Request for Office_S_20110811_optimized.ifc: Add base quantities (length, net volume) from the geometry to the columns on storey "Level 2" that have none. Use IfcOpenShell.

First a look at what the model holds.

```python
import ifcopenshell
import ifcopenshell.util.element
import ifcopenshell.util.unit

model = ifcopenshell.open("Office_S_20110811_optimized.ifc")
print(model.schema)
for unit_type in ("LENGTHUNIT", "AREAUNIT", "VOLUMEUNIT"):
    print(unit_type, ifcopenshell.util.unit.calculate_unit_scale(model, unit_type))
storey = next(s for s in model.by_type("IfcBuildingStorey") if s.Name == "Level 2")
columns = [e for e in ifcopenshell.util.element.get_decomposition(storey) if e.is_a("IfcColumn")]
for e in sorted(columns, key=lambda e: e.id()):
    print(e.id(), e.is_a(), e.Name, list(ifcopenshell.util.element.get_psets(e, qtos_only=True)), sep=" | ")
```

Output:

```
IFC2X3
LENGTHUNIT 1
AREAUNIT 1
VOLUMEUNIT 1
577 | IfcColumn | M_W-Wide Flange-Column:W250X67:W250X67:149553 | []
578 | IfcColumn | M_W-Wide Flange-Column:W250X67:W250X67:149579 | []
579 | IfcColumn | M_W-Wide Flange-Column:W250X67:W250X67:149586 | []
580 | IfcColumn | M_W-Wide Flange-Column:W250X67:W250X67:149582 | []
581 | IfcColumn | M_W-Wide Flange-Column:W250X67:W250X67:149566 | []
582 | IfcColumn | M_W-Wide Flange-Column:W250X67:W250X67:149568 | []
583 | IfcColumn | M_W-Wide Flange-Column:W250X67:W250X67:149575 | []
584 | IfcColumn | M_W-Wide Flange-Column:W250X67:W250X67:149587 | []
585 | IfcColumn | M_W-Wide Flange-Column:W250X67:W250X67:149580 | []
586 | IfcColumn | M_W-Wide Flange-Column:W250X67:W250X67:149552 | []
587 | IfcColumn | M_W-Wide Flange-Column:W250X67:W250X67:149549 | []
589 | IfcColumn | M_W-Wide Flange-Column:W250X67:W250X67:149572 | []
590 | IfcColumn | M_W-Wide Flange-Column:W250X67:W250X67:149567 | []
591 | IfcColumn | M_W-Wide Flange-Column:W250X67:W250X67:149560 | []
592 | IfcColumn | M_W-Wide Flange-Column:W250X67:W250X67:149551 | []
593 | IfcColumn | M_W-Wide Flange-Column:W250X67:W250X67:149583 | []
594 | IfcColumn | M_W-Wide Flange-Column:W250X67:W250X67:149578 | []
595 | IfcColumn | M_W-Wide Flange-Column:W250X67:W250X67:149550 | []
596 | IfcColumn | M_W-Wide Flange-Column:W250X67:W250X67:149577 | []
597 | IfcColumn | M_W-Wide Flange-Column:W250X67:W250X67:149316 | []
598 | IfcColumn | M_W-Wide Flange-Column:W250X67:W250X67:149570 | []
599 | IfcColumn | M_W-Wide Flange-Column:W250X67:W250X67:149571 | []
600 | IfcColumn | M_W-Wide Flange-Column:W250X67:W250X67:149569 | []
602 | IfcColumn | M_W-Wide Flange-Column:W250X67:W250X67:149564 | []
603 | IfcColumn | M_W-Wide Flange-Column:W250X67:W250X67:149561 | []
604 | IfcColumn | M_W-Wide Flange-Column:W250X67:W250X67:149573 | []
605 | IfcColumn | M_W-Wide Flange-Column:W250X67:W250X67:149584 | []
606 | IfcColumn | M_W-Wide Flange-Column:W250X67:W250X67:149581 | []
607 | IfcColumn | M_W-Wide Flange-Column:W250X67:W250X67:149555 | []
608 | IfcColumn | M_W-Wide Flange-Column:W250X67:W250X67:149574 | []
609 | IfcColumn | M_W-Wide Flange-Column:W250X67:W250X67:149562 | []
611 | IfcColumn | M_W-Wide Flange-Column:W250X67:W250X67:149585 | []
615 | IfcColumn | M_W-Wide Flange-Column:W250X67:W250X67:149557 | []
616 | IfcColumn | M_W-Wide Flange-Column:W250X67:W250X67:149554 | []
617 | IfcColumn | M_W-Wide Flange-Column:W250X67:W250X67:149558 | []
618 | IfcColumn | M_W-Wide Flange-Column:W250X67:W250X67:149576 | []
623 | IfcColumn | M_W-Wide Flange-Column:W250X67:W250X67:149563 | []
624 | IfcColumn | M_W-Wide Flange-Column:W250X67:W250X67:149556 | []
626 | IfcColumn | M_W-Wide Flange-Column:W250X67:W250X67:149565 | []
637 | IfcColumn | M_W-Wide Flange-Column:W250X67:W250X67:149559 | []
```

```python
import ifcopenshell
import ifcopenshell.api.pset
import ifcopenshell.geom
import ifcopenshell.util.element
import ifcopenshell.util.shape
import ifcopenshell.util.unit

model = ifcopenshell.open("Office_S_20110811_optimized.ifc")
unit_scale = ifcopenshell.util.unit.calculate_unit_scale(model)
volume_scale = ifcopenshell.util.unit.calculate_unit_scale(model, "VOLUMEUNIT")
settings = ifcopenshell.geom.settings()

storey = next(s for s in model.by_type("IfcBuildingStorey") if s.Name == "Level 2")
columns = [e for e in ifcopenshell.util.element.get_decomposition(storey) if e.is_a("IfcColumn")]

for e in sorted(columns, key=lambda e: e.id()):
    if ifcopenshell.util.element.get_psets(e, qtos_only=True, should_inherit=False):
        continue
    # Geometry comes back in metres, in the element's own axes.
    shape = ifcopenshell.geom.create_shape(settings, e)
    values = {
        "Length": ifcopenshell.util.shape.get_z(shape.geometry) / unit_scale,
        "NetVolume": ifcopenshell.util.shape.get_volume(shape.geometry) / volume_scale,
    }
    qto = ifcopenshell.api.pset.add_qto(model, product=e, name="BaseQuantities")
    ifcopenshell.api.pset.edit_qto(model, qto=qto, properties=values)
    print(e.id(), {k: round(v, 3) for k, v in values.items()})

model.write("Office_S_20110811_optimized-out.ifc")
```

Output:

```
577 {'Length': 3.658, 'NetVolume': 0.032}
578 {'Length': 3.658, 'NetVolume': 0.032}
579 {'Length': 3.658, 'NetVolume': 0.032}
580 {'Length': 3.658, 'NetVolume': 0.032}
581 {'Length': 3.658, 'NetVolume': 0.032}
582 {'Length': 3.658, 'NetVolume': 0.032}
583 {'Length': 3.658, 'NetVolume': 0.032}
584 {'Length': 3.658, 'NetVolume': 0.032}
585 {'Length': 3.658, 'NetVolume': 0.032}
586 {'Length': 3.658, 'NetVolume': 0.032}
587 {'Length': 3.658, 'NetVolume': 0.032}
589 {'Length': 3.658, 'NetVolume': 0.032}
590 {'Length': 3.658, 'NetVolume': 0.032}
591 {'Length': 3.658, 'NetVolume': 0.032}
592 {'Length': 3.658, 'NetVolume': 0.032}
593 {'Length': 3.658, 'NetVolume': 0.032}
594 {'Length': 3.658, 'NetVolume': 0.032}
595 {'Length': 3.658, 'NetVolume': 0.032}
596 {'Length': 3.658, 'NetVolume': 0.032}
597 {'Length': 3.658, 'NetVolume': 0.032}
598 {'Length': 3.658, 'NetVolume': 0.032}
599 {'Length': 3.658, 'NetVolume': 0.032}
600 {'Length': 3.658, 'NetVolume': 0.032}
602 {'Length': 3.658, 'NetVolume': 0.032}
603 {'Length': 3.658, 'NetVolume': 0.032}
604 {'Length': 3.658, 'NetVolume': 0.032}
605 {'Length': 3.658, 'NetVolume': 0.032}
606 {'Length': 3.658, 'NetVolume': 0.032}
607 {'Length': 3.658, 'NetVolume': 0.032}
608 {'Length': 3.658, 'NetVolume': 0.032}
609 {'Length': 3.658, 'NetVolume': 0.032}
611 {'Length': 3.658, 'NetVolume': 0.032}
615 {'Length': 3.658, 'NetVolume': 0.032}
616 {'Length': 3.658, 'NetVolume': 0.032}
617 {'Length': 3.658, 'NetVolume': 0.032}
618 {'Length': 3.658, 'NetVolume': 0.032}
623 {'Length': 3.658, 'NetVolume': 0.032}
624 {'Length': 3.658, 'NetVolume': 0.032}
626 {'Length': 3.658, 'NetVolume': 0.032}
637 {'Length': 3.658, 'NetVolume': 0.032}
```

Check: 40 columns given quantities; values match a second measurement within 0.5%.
